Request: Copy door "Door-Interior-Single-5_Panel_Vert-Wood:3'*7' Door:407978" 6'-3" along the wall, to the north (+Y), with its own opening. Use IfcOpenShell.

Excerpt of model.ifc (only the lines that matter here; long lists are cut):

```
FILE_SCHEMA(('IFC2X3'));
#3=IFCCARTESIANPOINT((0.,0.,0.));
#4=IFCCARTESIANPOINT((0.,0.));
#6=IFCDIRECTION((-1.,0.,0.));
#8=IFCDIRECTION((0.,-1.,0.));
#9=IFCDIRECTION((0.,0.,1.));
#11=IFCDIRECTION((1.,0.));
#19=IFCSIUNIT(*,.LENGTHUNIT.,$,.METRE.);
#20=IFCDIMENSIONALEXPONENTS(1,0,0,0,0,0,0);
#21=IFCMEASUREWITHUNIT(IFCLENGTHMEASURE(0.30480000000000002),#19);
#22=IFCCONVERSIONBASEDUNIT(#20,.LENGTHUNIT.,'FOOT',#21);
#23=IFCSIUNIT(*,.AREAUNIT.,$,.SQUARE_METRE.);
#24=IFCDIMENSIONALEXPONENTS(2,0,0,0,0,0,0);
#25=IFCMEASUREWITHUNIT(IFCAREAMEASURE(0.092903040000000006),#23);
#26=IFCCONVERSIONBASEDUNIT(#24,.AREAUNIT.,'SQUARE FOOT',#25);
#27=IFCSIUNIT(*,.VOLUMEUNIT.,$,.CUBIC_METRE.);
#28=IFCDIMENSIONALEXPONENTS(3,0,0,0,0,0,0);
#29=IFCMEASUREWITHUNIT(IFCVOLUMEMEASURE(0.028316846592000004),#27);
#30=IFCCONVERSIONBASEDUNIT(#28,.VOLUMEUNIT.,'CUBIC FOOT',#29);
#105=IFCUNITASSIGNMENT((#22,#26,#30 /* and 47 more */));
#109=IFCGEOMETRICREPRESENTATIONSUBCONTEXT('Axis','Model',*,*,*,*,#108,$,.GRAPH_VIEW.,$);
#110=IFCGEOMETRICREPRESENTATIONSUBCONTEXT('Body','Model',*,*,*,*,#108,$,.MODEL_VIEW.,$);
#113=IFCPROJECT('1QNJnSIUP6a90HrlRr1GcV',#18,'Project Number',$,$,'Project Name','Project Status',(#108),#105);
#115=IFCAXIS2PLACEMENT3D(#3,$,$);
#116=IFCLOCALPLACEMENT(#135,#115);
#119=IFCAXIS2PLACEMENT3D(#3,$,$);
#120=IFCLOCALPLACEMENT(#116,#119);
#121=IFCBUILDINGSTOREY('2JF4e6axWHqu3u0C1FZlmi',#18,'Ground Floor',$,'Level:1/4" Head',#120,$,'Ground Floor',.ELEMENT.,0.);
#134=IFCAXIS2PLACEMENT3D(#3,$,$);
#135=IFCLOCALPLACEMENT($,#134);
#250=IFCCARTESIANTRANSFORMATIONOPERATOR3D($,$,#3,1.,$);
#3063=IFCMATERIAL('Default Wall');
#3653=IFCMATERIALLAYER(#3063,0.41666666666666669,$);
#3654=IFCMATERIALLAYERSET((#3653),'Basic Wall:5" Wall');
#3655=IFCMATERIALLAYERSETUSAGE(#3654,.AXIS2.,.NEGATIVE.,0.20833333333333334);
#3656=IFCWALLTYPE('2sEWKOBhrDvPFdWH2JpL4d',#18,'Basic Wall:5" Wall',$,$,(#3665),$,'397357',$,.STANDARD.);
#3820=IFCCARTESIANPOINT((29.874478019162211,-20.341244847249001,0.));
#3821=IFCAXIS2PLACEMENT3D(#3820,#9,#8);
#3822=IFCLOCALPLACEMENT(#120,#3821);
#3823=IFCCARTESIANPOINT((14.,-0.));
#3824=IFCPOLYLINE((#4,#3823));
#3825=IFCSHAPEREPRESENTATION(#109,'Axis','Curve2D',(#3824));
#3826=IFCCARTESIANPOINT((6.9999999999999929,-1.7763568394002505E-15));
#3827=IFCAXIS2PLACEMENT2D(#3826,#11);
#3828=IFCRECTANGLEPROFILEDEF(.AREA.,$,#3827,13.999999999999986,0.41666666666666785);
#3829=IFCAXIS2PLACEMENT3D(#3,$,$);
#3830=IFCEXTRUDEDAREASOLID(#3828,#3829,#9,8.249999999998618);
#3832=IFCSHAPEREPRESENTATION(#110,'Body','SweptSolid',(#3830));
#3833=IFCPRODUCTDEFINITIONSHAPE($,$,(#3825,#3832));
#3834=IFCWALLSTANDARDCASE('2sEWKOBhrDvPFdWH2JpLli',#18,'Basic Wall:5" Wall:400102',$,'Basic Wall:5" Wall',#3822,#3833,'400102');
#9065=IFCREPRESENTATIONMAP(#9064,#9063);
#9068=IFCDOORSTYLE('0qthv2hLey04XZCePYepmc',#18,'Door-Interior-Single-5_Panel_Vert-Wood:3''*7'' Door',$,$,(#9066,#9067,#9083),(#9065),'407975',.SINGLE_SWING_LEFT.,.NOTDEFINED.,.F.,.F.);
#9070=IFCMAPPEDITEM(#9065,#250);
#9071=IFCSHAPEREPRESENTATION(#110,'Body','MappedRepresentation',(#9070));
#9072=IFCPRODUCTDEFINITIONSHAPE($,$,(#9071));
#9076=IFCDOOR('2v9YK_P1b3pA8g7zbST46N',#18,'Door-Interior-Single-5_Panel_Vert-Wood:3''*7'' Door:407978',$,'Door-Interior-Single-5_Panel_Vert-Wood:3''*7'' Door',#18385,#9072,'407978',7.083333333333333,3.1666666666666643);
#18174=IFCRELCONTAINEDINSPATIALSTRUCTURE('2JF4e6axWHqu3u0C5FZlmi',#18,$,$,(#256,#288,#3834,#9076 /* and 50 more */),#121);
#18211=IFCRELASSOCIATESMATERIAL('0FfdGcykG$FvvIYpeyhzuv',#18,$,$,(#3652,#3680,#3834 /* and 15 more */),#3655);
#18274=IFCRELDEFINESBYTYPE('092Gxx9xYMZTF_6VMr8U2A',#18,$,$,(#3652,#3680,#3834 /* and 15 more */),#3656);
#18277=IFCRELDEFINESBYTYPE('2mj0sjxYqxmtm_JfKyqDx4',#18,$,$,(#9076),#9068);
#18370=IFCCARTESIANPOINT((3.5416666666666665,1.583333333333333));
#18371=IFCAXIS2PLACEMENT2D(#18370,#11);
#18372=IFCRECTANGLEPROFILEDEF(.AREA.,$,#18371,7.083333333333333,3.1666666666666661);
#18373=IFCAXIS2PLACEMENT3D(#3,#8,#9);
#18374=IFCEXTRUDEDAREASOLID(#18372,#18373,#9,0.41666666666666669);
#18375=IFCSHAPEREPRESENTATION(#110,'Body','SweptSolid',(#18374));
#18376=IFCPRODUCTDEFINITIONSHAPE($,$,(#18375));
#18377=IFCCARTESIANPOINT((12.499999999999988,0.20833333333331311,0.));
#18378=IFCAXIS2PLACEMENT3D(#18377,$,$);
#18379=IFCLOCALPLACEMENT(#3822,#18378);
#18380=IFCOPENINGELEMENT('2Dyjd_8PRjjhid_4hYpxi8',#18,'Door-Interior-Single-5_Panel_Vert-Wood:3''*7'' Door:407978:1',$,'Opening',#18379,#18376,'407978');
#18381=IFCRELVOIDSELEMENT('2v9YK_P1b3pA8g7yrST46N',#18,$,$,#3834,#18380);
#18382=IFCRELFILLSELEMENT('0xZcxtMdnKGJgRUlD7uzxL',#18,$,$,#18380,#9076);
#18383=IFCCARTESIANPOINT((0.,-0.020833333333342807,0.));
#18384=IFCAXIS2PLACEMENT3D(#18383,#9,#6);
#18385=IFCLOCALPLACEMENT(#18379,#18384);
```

```python
import ifcopenshell
import ifcopenshell.api.feature
import ifcopenshell.api.geometry
import ifcopenshell.api.root
import ifcopenshell.geom
import ifcopenshell.util.element
import ifcopenshell.util.placement
import ifcopenshell.util.shape
import ifcopenshell.util.unit

model = ifcopenshell.open("model.ifc")
unit_scale = ifcopenshell.util.unit.calculate_unit_scale(model)
settings = ifcopenshell.geom.settings()


def volume(element):
    """Net volume in cubic metres, openings subtracted."""
    shape = ifcopenshell.geom.create_shape(settings, element)
    return ifcopenshell.util.shape.get_volume(shape.geometry)


def reuse_history(source, copy):
    """copy_class also copies each property set's owner history, people and application; keep the originals."""
    for rel in copy.IsDefinedBy:
        if rel.is_a("IfcRelDefinesByProperties") and (history := rel.RelatingPropertyDefinition.OwnerHistory):
            rel.RelatingPropertyDefinition.OwnerHistory = source.OwnerHistory
            ifcopenshell.util.element.remove_deep2(model, history)


door = model.by_guid("2v9YK_P1b3pA8g7zbST46N")
opening = door.FillsVoids[0].RelatingOpeningElement
wall = opening.VoidsElements[0].RelatingBuildingElement
before = volume(wall)
shift = ifcopenshell.util.placement.get_local_placement(wall.ObjectPlacement)[:3, 0] * -75 * 0.0254 / unit_scale

# copy_class copies the void relationship, type, container and properties, but no geometry.
new_opening = ifcopenshell.api.root.copy_class(model, product=opening)
new_opening.Representation = ifcopenshell.util.element.copy_deep(
    model, opening.Representation, exclude=["IfcGeometricRepresentationContext", "IfcRepresentationMap"]
)
new_opening.Name = "Door-Interior-Single-5_Panel_Vert-Wood:3'*7' Door"
new_opening.Tag = None
new_door = ifcopenshell.api.root.copy_class(model, product=door)
new_door.Representation = ifcopenshell.util.element.copy_deep(
    model, door.Representation, exclude=["IfcGeometricRepresentationContext", "IfcRepresentationMap"]
)
new_door.Name = "Door-Interior-Single-5_Panel_Vert-Wood:3'*7' Door"
new_door.Tag = None
reuse_history(door, new_door)
fills = ifcopenshell.api.feature.add_filling(model, opening=new_opening, element=new_door)
fills.OwnerHistory = new_door.OwnerHistory  # required in IFC2X3

for old, new in ((opening, new_opening), (door, new_door)):
    matrix = ifcopenshell.util.placement.get_local_placement(old.ObjectPlacement)
    matrix[:3, 3] += shift
    ifcopenshell.api.geometry.edit_object_placement(model, product=new, matrix=matrix, is_si=False)

after = volume(wall)

print(f"wall volume {before:.3f} -> {after:.3f} m3")

model.write("model_edited.ifc")
```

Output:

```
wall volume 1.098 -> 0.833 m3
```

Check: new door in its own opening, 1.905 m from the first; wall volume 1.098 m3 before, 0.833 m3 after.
